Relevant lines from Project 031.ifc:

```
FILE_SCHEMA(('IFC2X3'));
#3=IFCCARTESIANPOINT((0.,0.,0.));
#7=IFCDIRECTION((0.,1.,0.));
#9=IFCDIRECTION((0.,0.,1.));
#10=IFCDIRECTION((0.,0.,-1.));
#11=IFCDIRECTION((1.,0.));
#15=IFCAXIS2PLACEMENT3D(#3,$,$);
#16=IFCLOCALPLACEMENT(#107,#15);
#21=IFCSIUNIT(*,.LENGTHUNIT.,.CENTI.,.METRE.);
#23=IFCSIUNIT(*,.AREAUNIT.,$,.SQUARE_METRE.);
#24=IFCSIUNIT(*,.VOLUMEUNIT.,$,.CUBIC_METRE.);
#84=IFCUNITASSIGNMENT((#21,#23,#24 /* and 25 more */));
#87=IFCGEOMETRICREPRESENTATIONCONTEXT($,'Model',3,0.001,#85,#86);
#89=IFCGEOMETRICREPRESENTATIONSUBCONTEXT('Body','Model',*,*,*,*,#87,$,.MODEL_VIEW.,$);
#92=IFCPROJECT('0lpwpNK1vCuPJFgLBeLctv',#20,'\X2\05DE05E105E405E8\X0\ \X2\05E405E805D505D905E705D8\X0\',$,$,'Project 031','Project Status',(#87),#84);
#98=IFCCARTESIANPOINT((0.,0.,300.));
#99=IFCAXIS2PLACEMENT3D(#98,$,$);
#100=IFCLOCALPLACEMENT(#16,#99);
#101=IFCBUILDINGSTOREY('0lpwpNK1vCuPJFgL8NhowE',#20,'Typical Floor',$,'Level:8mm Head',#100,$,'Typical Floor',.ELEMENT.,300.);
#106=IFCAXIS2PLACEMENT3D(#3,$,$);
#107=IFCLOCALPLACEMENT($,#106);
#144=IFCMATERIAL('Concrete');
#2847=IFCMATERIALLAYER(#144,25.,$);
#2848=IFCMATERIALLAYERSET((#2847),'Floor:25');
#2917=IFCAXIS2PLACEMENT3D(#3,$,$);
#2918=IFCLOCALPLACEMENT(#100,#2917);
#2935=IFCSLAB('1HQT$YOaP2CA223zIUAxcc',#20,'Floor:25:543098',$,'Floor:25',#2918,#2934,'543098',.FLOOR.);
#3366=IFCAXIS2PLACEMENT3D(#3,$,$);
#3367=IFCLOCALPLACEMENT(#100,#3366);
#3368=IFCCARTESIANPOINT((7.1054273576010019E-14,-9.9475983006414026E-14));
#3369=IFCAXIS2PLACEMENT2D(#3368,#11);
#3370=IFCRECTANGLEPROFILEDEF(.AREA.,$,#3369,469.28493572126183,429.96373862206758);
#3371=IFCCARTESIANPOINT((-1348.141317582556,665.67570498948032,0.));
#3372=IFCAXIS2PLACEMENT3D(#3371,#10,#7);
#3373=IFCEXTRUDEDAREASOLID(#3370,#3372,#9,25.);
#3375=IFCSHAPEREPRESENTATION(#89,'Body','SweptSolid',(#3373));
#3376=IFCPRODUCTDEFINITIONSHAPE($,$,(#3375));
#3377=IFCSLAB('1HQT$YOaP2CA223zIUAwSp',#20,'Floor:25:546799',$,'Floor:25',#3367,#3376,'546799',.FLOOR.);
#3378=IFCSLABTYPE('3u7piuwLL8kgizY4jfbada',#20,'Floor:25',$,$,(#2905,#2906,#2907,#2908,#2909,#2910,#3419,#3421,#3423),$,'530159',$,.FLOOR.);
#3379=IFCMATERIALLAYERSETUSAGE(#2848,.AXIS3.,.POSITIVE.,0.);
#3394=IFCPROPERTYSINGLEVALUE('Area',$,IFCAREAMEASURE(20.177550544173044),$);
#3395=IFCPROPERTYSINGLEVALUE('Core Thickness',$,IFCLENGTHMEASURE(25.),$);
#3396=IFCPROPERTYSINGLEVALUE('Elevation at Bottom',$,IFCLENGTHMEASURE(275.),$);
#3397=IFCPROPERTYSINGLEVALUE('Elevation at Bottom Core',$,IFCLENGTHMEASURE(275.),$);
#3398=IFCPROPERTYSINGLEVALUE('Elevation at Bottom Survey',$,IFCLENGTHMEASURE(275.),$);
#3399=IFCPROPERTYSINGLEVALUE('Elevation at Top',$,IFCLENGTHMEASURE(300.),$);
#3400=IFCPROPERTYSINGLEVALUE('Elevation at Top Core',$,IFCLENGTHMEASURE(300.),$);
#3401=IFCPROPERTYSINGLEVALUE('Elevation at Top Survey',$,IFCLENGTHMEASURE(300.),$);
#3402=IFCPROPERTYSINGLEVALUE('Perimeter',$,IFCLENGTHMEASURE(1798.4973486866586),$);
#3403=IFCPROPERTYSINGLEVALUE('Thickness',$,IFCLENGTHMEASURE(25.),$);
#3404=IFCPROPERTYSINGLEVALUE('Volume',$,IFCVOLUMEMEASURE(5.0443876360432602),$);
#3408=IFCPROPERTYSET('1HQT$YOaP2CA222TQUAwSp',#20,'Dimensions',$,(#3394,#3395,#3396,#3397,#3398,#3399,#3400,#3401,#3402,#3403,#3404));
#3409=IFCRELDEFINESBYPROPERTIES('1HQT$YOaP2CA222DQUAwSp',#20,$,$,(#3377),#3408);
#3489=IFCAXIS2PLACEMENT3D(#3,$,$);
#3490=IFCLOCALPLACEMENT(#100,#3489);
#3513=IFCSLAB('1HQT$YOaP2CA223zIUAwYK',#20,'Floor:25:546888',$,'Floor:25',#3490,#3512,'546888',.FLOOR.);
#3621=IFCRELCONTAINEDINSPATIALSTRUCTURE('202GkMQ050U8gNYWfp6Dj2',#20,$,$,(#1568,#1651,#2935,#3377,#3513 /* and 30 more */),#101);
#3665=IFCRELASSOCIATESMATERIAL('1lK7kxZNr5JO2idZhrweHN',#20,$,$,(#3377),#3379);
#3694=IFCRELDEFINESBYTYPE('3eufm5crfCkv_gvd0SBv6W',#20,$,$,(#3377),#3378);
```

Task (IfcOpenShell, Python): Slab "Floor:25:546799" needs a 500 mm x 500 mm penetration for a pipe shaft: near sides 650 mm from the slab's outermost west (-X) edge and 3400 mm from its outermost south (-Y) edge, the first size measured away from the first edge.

```python
import numpy as np
import ifcopenshell
import ifcopenshell.api.feature
import ifcopenshell.api.geometry
import ifcopenshell.api.pset
import ifcopenshell.api.root
import ifcopenshell.geom
import ifcopenshell.util.element
import ifcopenshell.util.placement
import ifcopenshell.util.representation
import ifcopenshell.util.shape
import ifcopenshell.util.unit

model = ifcopenshell.open("Project 031.ifc")
unit_scale = ifcopenshell.util.unit.calculate_unit_scale(model)
area_scale = ifcopenshell.util.unit.calculate_unit_scale(model, "AREAUNIT")
volume_scale = ifcopenshell.util.unit.calculate_unit_scale(model, "VOLUMEUNIT")
settings = ifcopenshell.geom.settings()


def volume(element):
    """Net volume in cubic metres, openings subtracted."""
    shape = ifcopenshell.geom.create_shape(settings, element)
    return ifcopenshell.util.shape.get_volume(shape.geometry)


slab = model.by_guid("1HQT$YOaP2CA223zIUAwSp")
before = volume(slab)

# Extent in the slab's own axes, in metres. The edges named are its -X and -Y sides.
slab_shape = ifcopenshell.geom.create_shape(settings, slab)
vertices = ifcopenshell.util.shape.get_vertices(slab_shape.geometry)
x_min, y_min, bottom = vertices.min(axis=0)
top = vertices[:, 2].max()

opening = ifcopenshell.api.root.create_entity(model, ifc_class="IfcOpeningElement", name="Pipe shaft opening")
context = ifcopenshell.util.representation.get_context(model, "Model", "Body", "MODEL_VIEW")
width, depth = 0.5, 0.5
outline = [(0.0, 0.0), (width, 0.0), (width, depth), (0.0, depth), (0.0, 0.0)]
# Overshoot both faces by 50 mm so the cut is clean.
shape = ifcopenshell.api.geometry.add_slab_representation(
    model, context=context, depth=top - bottom + 0.1, polyline=outline
)
ifcopenshell.api.geometry.assign_representation(model, product=opening, representation=shape)

matrix = ifcopenshell.util.placement.get_local_placement(slab.ObjectPlacement)
matrix[:, 3] = matrix @ np.append(np.array([x_min + 0.65, y_min + 3.4, bottom - 0.05]) / unit_scale, 1.0)
ifcopenshell.api.geometry.edit_object_placement(model, product=opening, matrix=matrix, is_si=False)
ifcopenshell.api.feature.add_feature(model, feature=opening, element=slab)

after = volume(slab)

# Update the slab's stored quantities.
pset = model.by_id(ifcopenshell.util.element.get_pset(slab, "Dimensions", should_inherit=False)["id"])
ifcopenshell.api.pset.edit_pset(model, pset=pset, properties={
    "Area": model.create_entity("IfcAreaMeasure", after / (top - bottom) / area_scale),
    "Volume": model.create_entity("IfcVolumeMeasure", after / volume_scale),
})

print(f"slab volume {before:.3f} -> {after:.3f} m3")

model.write("Project 031_updated.ifc")
```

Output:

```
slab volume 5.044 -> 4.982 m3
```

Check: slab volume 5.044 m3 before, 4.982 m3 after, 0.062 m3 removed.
